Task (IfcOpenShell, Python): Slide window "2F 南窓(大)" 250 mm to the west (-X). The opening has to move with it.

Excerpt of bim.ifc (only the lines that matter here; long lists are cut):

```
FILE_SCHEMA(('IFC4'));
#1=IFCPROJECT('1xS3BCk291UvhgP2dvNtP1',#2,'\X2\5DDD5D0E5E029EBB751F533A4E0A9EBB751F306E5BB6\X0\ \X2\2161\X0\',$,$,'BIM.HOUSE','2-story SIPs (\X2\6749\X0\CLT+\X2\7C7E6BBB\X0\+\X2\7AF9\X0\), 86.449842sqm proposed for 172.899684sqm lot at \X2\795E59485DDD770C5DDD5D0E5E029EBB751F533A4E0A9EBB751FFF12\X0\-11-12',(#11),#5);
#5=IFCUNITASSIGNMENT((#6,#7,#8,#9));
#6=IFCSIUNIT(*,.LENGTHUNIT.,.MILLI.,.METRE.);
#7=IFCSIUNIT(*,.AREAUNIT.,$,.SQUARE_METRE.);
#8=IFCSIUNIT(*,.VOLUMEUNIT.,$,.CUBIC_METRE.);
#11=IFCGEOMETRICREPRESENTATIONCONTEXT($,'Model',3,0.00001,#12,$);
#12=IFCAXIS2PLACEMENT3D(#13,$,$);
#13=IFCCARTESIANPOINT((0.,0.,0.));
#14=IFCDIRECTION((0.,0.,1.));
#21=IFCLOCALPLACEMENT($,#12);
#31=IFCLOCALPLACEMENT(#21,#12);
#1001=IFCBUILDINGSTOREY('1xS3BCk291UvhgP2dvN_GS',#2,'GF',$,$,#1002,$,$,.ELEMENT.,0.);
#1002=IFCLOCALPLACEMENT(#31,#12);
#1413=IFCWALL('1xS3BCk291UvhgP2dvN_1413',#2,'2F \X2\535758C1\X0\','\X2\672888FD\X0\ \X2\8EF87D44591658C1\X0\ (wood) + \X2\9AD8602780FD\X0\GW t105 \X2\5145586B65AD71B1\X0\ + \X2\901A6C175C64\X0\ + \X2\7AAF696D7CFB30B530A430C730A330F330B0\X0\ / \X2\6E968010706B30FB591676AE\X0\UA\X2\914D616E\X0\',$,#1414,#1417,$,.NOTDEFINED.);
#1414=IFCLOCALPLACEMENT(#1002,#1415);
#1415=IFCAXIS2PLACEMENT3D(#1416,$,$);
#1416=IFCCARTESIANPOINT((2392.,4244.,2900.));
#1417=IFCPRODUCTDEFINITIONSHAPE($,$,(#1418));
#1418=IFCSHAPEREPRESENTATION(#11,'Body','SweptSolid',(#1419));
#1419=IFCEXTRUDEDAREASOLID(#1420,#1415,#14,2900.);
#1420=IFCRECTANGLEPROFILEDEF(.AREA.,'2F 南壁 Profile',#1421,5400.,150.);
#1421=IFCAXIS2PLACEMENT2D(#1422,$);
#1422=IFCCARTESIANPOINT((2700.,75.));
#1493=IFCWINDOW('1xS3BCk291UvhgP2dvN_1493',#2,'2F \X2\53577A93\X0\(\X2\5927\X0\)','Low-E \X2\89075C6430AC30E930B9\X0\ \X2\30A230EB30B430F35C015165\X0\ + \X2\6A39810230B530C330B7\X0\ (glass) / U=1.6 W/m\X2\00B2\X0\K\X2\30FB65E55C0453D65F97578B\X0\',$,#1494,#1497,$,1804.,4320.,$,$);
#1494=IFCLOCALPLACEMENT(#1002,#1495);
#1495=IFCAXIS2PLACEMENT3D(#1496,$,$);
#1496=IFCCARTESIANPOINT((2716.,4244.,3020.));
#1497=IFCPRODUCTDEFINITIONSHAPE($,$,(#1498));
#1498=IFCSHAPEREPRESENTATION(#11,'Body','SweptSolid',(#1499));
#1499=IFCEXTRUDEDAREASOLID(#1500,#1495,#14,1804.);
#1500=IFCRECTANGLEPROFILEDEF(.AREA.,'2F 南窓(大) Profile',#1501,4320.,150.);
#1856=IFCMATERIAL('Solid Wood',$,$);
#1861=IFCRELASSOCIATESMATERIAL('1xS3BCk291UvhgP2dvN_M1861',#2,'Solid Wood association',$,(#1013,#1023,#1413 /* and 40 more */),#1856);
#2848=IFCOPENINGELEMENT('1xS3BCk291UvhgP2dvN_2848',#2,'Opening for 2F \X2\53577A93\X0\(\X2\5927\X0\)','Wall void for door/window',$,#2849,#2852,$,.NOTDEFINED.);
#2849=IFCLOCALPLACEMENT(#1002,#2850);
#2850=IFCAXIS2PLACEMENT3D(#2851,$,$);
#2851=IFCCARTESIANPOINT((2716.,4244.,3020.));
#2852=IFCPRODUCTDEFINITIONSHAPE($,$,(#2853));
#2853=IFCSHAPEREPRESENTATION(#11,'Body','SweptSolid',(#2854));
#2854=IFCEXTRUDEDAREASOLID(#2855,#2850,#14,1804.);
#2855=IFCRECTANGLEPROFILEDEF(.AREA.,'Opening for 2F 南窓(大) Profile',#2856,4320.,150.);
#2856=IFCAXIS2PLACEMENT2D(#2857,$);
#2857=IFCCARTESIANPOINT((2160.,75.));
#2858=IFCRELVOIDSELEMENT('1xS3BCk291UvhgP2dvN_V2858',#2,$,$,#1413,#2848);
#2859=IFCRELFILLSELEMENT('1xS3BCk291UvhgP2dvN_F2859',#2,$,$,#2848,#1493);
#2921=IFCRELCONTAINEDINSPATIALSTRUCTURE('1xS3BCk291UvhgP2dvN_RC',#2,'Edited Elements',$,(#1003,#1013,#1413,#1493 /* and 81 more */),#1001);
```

```python
import ifcopenshell
import ifcopenshell.api.geometry
import ifcopenshell.util.placement

model = ifcopenshell.open("bim.ifc")

window = model.by_id(1493)
opening = window.FillsVoids[0].RelatingOpeningElement
wall = opening.VoidsElements[0].RelatingBuildingElement

wall_matrix = ifcopenshell.util.placement.get_local_placement(wall.ObjectPlacement)
shift = wall_matrix[:3, 0] * -250.0
before = ifcopenshell.util.placement.get_local_placement(window.ObjectPlacement)[:3, 3].copy()

# The window is not placed relative to its opening, so move both.
for product in (opening, window):
    matrix = ifcopenshell.util.placement.get_local_placement(product.ObjectPlacement)
    matrix[:3, 3] += shift
    ifcopenshell.api.geometry.edit_object_placement(model, product=product, matrix=matrix, is_si=False)

after = ifcopenshell.util.placement.get_local_placement(window.ObjectPlacement)[:3, 3]
print("window moved by", (after - before).round(3) + 0.0)

model.write("bim_edited.ifc")
```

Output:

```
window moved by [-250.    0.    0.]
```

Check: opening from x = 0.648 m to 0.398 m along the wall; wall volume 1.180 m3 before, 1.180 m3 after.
